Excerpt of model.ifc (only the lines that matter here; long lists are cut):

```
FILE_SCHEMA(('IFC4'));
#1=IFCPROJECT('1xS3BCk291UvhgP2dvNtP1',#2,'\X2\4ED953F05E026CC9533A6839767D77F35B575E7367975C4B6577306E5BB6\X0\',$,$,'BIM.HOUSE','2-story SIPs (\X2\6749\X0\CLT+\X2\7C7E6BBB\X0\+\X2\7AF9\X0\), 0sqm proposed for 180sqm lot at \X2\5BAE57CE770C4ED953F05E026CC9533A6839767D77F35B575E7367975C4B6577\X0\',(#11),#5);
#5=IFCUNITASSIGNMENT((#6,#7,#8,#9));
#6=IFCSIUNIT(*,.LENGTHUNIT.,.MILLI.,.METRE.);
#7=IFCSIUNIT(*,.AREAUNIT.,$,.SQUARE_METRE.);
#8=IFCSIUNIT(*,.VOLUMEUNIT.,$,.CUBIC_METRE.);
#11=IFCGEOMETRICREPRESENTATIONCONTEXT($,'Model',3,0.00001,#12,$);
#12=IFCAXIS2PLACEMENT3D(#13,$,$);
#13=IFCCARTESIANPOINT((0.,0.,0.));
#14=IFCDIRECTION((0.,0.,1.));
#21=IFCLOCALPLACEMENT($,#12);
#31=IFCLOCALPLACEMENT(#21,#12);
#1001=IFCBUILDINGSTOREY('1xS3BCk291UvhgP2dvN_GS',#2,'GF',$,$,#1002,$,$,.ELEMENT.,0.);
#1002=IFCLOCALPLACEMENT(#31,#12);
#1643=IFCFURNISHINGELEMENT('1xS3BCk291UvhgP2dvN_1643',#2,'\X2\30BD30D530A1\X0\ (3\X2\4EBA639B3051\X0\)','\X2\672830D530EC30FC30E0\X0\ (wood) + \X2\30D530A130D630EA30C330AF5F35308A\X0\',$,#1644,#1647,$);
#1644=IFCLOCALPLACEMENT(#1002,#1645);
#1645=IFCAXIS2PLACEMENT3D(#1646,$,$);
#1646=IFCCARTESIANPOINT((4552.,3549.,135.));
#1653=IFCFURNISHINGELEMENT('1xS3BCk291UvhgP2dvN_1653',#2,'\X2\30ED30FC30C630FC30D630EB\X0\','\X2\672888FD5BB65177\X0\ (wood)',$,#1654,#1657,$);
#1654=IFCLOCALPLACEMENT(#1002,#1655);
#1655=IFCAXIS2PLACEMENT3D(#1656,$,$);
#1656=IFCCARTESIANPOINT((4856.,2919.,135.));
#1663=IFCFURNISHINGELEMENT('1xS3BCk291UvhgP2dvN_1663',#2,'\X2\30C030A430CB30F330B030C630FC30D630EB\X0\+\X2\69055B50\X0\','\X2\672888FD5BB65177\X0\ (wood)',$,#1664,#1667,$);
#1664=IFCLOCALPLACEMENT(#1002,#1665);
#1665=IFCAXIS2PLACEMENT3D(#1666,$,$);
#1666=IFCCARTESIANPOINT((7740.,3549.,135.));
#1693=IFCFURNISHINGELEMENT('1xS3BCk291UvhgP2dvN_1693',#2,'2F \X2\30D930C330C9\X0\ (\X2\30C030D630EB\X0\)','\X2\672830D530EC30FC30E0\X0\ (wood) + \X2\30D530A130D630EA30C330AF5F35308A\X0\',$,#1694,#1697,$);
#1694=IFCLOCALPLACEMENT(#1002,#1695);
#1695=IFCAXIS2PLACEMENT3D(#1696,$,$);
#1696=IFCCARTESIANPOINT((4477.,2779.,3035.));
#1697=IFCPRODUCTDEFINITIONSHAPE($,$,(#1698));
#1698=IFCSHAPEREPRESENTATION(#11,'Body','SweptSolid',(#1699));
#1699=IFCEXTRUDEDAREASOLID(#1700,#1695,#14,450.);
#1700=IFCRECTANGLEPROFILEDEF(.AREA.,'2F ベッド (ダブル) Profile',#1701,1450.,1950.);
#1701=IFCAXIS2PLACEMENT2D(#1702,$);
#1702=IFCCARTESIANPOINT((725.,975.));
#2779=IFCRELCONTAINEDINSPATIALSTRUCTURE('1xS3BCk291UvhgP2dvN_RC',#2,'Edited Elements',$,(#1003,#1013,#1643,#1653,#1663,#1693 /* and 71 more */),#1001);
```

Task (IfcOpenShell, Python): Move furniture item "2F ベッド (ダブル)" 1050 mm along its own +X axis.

```python
import ifcopenshell
import ifcopenshell.api.geometry
import ifcopenshell.util.placement
import ifcopenshell.util.unit

model = ifcopenshell.open("model.ifc")
unit_scale = ifcopenshell.util.unit.calculate_unit_scale(model)

item = model.by_guid("1xS3BCk291UvhgP2dvN_1693")
matrix = ifcopenshell.util.placement.get_local_placement(item.ObjectPlacement)
matrix[:3, 3] += matrix[:3, 0] * 1.05 / unit_scale
ifcopenshell.api.geometry.edit_object_placement(model, product=item, matrix=matrix, is_si=False)

print(ifcopenshell.util.placement.get_local_placement(item.ObjectPlacement).round(3) + 0.0)

model.write("model_rev.ifc")
```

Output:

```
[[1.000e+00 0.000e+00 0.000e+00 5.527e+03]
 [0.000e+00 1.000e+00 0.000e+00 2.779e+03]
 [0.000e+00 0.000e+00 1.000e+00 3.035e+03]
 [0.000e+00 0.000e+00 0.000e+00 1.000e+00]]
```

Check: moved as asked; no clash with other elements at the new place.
